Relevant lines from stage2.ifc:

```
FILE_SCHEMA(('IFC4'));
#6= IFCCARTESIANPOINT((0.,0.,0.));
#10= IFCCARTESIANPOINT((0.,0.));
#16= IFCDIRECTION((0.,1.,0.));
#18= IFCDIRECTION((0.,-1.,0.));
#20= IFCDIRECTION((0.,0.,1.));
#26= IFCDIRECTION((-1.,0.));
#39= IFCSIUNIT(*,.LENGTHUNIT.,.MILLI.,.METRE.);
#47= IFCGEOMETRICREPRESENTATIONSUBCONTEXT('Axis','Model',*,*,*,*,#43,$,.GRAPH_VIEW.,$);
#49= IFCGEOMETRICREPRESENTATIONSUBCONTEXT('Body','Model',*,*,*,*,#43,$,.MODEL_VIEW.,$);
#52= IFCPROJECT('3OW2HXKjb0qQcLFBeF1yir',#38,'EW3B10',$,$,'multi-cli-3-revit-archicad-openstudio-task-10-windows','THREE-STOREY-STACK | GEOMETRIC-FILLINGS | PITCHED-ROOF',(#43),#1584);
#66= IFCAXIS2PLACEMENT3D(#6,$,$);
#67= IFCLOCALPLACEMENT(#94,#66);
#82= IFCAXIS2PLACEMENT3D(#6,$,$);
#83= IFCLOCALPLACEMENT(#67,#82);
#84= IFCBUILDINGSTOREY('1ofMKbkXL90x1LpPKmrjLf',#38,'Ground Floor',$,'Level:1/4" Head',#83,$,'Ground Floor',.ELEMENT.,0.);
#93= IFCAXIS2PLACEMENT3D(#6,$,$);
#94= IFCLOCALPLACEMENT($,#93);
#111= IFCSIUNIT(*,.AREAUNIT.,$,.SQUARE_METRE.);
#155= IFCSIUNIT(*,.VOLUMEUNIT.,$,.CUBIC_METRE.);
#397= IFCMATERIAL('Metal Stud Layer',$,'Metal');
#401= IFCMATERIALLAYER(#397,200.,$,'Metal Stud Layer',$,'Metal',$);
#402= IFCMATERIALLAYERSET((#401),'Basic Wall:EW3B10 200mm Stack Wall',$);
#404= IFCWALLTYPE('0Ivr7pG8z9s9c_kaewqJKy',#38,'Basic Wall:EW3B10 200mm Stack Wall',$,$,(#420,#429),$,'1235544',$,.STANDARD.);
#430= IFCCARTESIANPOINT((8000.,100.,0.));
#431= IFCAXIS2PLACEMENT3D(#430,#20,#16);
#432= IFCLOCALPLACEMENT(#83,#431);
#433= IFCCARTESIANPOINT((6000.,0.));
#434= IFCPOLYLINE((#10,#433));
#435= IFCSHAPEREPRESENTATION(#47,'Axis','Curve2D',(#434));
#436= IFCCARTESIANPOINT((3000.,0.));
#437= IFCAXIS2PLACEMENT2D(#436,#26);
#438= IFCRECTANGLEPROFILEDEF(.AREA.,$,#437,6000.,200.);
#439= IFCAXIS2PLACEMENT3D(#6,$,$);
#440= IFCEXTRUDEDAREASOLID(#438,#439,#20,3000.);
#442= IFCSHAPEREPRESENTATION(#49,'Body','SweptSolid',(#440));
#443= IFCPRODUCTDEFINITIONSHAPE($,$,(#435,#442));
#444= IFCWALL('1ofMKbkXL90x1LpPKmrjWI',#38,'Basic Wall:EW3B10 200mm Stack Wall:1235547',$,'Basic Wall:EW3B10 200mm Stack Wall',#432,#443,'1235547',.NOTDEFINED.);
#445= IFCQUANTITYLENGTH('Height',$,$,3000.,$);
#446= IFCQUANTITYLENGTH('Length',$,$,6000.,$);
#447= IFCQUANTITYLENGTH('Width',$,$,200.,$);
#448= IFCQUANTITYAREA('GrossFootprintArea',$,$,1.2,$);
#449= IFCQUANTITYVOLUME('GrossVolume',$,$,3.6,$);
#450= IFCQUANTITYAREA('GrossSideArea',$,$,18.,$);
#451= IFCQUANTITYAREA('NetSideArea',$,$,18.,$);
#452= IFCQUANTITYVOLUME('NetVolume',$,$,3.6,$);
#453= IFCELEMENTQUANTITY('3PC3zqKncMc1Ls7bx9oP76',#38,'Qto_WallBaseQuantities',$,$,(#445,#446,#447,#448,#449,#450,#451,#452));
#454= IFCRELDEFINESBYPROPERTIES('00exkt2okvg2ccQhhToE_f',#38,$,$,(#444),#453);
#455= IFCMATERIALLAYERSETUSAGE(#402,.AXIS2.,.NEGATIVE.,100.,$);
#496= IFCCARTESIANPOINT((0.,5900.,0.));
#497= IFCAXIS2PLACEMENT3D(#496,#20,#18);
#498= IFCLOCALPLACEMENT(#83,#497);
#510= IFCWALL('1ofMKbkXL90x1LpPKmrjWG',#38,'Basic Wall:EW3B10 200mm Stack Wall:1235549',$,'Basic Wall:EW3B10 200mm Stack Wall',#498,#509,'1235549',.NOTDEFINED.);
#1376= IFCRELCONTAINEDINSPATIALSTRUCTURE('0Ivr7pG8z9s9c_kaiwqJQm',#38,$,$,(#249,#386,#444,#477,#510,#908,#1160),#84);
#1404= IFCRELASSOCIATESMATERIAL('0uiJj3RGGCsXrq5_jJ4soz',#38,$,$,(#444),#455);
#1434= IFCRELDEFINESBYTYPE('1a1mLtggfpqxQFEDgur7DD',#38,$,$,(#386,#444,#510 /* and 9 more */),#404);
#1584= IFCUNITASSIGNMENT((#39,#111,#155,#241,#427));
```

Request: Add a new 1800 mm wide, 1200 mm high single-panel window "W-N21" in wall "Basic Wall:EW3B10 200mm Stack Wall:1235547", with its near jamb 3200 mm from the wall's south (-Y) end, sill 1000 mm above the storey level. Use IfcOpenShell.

```python
import numpy as np
import ifcopenshell
import ifcopenshell.api.feature
import ifcopenshell.api.geometry
import ifcopenshell.api.pset
import ifcopenshell.api.root
import ifcopenshell.api.spatial
import ifcopenshell.geom
import ifcopenshell.util.element
import ifcopenshell.util.placement
import ifcopenshell.util.representation
import ifcopenshell.util.shape
import ifcopenshell.util.unit

model = ifcopenshell.open("stage2.ifc")
unit_scale = ifcopenshell.util.unit.calculate_unit_scale(model)
area_scale = ifcopenshell.util.unit.calculate_unit_scale(model, "AREAUNIT")
volume_scale = ifcopenshell.util.unit.calculate_unit_scale(model, "VOLUMEUNIT")
settings = ifcopenshell.geom.settings()


def volume(element):
    """Net volume in cubic metres, openings subtracted."""
    shape = ifcopenshell.geom.create_shape(settings, element)
    return ifcopenshell.util.shape.get_volume(shape.geometry)


wall = model.by_guid("1ofMKbkXL90x1LpPKmrjWI")
storey = ifcopenshell.util.element.get_container(wall, ifc_class="IfcBuildingStorey")
context = ifcopenshell.util.representation.get_context(model, "Model", "Body", "MODEL_VIEW")
before = volume(wall)

width, height, from_end, sill = 1.8, 1.2, 3.2, 1  # metres

# The wall runs along its own X axis, and the end named is its -X end.
wall_shape = ifcopenshell.geom.create_shape(settings, wall)
x, y, z = ifcopenshell.util.shape.get_vertices(wall_shape.geometry).T
start = x.min() + from_end
face, thickness = float(y.min()), float(y.max() - y.min())
wall_matrix = ifcopenshell.util.placement.get_local_placement(wall.ObjectPlacement)
level = ifcopenshell.util.placement.get_local_placement(storey.ObjectPlacement)[2, 3]


def in_wall(x, y):
    """Placement at x, y metres in the wall's axes, at sill height."""
    matrix = wall_matrix.copy()
    matrix[:, 3] = wall_matrix @ np.array([x / unit_scale, y / unit_scale, 0.0, 1.0])
    matrix[2, 3] = level + sill / unit_scale
    return matrix


# Opening: a box that overshoots both wall faces by 50 mm.
opening = ifcopenshell.api.root.create_entity(model, ifc_class="IfcOpeningElement", predefined_type="OPENING")
box = ifcopenshell.api.geometry.add_wall_representation(
    model, context=context, length=width, height=height, thickness=thickness + 0.1
)
ifcopenshell.api.geometry.assign_representation(model, product=opening, representation=box)
ifcopenshell.api.geometry.edit_object_placement(model, product=opening, matrix=in_wall(start, face - 0.05), is_si=False)
ifcopenshell.api.feature.add_feature(model, feature=opening, element=wall)

window = ifcopenshell.api.root.create_entity(model, ifc_class="IfcWindow", name="W-N21", predefined_type="WINDOW")
window.OverallWidth, window.OverallHeight = width / unit_scale, height / unit_scale
window.PartitioningType = "SINGLE_PANEL"
body = ifcopenshell.api.geometry.add_window_representation(
    model,
    context=context,
    overall_width=window.OverallWidth,
    overall_height=window.OverallHeight,
    partition_type="SINGLE_PANEL",
)
ifcopenshell.api.geometry.assign_representation(model, product=window, representation=body)
ifcopenshell.api.spatial.assign_container(model, products=[window], relating_structure=storey)
ifcopenshell.api.feature.add_filling(model, opening=opening, element=window)

# Centre the window in the wall's thickness.
ifcopenshell.api.geometry.edit_object_placement(model, product=window, matrix=in_wall(start, face), is_si=False)
window_shape = ifcopenshell.geom.create_shape(settings, window)
depth = ifcopenshell.util.shape.get_vertices(window_shape.geometry)[:, 1]
offset = face + thickness / 2 - (depth.min() + depth.max()) / 2
ifcopenshell.api.geometry.edit_object_placement(model, product=window, matrix=in_wall(start, offset), is_si=False)

after = volume(wall)

# Update the wall's stored quantities.
qto = model.by_id(ifcopenshell.util.element.get_pset(wall, "Qto_WallBaseQuantities", should_inherit=False)["id"])
ifcopenshell.api.pset.edit_qto(model, qto=qto, properties={
    "NetSideArea": after / thickness / area_scale,
    "NetVolume": after / volume_scale,
})

print(f"wall volume {before:.3f} -> {after:.3f} m3")

model.write("stage2_edited.ifc")
```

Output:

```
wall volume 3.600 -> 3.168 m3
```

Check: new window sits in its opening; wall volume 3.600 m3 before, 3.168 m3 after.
